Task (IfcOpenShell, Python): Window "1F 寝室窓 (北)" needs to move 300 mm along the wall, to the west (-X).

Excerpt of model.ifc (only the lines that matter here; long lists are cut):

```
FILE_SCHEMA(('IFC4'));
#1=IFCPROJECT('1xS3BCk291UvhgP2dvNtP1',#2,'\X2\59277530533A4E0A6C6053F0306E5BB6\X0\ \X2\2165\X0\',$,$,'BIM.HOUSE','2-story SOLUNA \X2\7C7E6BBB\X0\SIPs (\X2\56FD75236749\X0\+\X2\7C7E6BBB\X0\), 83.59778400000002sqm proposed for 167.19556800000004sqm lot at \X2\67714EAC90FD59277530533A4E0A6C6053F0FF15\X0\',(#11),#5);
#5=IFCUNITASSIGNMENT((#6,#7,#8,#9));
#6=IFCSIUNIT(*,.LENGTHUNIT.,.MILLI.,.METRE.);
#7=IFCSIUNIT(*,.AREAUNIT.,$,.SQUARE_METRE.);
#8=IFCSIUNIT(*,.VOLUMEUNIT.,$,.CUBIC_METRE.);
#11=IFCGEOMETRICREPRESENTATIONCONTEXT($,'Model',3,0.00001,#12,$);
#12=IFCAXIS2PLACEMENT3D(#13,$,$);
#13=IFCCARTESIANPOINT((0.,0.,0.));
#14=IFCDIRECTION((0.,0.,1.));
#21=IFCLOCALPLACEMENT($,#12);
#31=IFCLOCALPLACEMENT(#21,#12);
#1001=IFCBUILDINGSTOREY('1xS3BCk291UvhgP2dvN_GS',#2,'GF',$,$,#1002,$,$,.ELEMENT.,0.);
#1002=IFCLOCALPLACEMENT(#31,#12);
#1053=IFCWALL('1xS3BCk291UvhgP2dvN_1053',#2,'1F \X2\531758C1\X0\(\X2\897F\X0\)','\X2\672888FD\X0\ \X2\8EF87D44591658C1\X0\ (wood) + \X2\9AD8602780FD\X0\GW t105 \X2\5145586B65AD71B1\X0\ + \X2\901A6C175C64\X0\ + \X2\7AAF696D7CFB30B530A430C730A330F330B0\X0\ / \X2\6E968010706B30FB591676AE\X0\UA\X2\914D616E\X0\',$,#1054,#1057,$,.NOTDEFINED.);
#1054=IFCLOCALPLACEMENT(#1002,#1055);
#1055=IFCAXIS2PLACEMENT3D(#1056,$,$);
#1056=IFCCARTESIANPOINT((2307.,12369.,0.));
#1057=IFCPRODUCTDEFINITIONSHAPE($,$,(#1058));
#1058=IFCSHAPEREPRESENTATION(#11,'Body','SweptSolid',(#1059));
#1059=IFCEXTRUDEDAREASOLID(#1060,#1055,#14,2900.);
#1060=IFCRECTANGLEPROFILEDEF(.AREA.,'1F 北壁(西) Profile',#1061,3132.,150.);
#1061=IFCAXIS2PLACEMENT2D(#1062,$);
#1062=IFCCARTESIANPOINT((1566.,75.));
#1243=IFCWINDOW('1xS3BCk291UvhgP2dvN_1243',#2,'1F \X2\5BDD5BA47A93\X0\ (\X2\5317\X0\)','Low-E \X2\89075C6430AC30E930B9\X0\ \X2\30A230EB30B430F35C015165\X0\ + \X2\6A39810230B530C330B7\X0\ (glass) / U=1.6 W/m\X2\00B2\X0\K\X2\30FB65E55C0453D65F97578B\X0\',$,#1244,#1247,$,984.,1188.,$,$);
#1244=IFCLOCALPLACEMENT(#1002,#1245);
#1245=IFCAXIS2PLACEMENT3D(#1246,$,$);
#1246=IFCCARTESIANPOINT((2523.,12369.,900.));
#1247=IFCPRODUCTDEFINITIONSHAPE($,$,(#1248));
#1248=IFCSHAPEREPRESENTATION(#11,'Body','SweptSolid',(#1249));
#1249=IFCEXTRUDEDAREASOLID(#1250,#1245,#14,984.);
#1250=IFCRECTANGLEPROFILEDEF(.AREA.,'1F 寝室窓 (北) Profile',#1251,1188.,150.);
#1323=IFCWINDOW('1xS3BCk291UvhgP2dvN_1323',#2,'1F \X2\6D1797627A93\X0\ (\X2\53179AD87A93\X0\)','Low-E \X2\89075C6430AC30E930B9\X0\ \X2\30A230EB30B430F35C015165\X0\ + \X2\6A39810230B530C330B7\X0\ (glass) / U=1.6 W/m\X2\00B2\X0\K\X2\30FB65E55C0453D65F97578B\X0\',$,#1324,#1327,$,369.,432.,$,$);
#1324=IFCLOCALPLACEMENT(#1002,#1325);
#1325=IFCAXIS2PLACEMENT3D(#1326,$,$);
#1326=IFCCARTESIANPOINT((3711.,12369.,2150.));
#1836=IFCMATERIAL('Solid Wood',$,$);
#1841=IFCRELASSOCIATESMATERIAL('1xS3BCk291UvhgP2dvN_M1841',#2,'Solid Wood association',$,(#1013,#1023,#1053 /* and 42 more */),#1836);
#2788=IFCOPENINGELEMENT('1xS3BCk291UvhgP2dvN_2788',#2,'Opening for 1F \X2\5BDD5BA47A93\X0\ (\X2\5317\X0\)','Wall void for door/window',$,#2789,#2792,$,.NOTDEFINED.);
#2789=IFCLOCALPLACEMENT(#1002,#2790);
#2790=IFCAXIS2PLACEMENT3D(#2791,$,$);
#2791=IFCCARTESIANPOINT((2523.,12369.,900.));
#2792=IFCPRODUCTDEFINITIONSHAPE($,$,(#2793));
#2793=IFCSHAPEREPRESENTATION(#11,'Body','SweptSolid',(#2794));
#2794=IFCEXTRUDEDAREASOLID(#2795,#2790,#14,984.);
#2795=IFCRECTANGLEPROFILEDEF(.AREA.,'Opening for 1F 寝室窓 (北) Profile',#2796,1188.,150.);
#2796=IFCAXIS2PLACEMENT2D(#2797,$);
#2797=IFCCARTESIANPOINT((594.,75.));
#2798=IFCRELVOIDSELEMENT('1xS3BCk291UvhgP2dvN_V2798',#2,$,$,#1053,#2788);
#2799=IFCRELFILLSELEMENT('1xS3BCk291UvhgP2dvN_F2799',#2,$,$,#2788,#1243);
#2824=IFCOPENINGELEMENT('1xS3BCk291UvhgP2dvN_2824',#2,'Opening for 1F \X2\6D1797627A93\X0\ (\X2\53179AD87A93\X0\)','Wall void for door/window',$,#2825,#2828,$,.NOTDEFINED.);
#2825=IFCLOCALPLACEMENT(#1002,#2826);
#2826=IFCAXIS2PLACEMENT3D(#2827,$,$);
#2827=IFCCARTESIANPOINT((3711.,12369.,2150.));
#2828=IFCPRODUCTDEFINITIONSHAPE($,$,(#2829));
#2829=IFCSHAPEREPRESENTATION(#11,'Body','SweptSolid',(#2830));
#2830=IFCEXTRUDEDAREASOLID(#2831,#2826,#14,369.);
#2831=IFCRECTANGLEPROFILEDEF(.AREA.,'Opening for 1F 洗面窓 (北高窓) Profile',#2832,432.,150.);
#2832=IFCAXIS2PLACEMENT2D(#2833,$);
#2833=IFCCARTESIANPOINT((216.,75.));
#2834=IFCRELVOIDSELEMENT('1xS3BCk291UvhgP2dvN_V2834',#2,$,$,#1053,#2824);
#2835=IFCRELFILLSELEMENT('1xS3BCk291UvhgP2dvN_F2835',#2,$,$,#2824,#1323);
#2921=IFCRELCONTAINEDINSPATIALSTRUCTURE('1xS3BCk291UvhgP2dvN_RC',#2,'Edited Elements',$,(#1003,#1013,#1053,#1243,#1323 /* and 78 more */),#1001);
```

```python
import ifcopenshell
import ifcopenshell.api.geometry
import ifcopenshell.util.placement
import ifcopenshell.util.unit

model = ifcopenshell.open("model.ifc")
unit_scale = ifcopenshell.util.unit.calculate_unit_scale(model)

window = model.by_guid("1xS3BCk291UvhgP2dvN_1243")
opening = window.FillsVoids[0].RelatingOpeningElement
wall = opening.VoidsElements[0].RelatingBuildingElement

wall_matrix = ifcopenshell.util.placement.get_local_placement(wall.ObjectPlacement)
shift = wall_matrix[:3, 0] * -0.3 / unit_scale
before = ifcopenshell.util.placement.get_local_placement(window.ObjectPlacement)[:3, 3].copy()

# The window is not placed relative to its opening, so move both.
for product in (opening, window):
    matrix = ifcopenshell.util.placement.get_local_placement(product.ObjectPlacement)
    matrix[:3, 3] += shift
    ifcopenshell.api.geometry.edit_object_placement(model, product=product, matrix=matrix, is_si=False)

after = ifcopenshell.util.placement.get_local_placement(window.ObjectPlacement)[:3, 3]
print("window moved by", (after - before).round(3) + 0.0)

model.write("model-out.ifc")
```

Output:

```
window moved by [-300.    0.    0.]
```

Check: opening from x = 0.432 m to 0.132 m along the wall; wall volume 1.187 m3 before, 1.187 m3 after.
